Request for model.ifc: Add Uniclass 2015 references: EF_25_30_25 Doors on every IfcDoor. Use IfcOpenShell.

First a look at what the model holds.

```python
import ifcopenshell

model = ifcopenshell.open("model.ifc")
print(model.schema)
print("classifications:", [c.Name for c in model.by_type("IfcClassification")])
for ifc_class in ("IfcDoor", "IfcRoof", "IfcStair", "IfcWall", "IfcWindow"):
    print(ifc_class, len(model.by_type(ifc_class)))
```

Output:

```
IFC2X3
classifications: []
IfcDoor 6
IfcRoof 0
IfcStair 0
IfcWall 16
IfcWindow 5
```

```python
import ifcopenshell
import ifcopenshell.api.classification

model = ifcopenshell.open("model.ifc")

# IFC2X3 requires Source and Edition and has no link from the project to the system.
system = model.create_entity("IfcClassification", Source="NBS", Edition="2015", Name="Uniclass 2015")

codes = {
    "IfcDoor": ("EF_25_30_25", "Doors"),
}
for ifc_class, (code, name) in codes.items():
    products = model.by_type(ifc_class)
    ifcopenshell.api.classification.add_reference(
        model, products=products, classification=system, identification=code, name=name
    )
    print(code, len(products))

model.write("model_edited.ifc")
```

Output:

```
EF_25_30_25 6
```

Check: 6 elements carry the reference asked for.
